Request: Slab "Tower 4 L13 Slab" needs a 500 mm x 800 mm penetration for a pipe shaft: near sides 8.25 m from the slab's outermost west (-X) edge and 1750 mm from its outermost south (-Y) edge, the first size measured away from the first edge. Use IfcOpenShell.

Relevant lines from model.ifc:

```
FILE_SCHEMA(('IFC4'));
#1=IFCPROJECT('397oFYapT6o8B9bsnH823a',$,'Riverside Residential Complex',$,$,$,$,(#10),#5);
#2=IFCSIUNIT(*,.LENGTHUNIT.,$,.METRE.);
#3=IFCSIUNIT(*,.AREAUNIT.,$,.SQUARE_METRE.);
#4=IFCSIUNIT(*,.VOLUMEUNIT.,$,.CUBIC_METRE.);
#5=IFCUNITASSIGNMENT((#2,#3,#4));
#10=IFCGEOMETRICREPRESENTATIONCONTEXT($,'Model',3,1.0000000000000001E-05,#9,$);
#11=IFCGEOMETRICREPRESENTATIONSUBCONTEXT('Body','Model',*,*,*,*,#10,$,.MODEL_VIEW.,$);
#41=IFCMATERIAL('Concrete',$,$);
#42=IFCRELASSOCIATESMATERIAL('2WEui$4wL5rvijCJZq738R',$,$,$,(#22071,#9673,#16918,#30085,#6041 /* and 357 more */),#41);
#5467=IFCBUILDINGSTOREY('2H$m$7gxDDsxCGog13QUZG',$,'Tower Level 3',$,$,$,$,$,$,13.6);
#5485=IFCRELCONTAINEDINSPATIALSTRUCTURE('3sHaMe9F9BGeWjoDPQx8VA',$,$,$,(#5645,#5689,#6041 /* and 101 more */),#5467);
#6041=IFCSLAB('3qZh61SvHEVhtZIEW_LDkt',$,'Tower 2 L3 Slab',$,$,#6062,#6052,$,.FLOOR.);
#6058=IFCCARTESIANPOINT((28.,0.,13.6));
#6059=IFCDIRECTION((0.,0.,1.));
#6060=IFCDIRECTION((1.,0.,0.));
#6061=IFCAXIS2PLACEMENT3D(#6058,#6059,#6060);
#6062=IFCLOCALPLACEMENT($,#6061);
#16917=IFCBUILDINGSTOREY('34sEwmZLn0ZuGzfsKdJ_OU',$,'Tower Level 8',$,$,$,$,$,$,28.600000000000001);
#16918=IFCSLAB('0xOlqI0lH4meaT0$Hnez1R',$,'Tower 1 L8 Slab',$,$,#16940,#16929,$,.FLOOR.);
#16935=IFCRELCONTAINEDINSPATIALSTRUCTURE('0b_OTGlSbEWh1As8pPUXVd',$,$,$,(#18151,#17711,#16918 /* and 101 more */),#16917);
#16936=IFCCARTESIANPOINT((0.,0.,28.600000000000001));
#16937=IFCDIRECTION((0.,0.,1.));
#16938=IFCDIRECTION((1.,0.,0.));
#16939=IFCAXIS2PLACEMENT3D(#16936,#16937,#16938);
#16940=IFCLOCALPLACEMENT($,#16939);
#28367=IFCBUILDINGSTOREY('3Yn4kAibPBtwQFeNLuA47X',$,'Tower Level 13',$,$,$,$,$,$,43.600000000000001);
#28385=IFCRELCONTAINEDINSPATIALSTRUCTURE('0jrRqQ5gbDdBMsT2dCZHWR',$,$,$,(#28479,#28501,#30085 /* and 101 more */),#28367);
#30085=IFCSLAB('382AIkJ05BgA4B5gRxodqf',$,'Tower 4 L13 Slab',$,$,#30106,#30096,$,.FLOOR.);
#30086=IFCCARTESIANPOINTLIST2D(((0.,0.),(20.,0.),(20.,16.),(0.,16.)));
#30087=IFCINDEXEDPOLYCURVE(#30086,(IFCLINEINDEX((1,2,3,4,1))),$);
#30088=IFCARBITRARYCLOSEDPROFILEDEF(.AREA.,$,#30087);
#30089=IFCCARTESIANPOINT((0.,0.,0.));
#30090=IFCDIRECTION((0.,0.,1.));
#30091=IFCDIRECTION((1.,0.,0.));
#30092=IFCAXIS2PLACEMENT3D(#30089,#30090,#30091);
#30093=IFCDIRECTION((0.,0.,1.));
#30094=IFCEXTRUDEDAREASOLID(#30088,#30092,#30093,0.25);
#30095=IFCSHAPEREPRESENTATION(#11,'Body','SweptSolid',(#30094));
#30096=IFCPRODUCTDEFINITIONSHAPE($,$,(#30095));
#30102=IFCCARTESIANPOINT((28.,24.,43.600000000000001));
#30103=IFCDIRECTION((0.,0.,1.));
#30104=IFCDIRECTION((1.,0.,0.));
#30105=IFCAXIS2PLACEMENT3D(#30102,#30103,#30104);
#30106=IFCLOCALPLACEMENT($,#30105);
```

```python
import numpy as np
import ifcopenshell
import ifcopenshell.api.feature
import ifcopenshell.api.geometry
import ifcopenshell.api.root
import ifcopenshell.geom
import ifcopenshell.util.placement
import ifcopenshell.util.representation
import ifcopenshell.util.shape
import ifcopenshell.util.unit

model = ifcopenshell.open("model.ifc")
unit_scale = ifcopenshell.util.unit.calculate_unit_scale(model)
settings = ifcopenshell.geom.settings()


def volume(element):
    """Net volume in cubic metres, openings subtracted."""
    shape = ifcopenshell.geom.create_shape(settings, element)
    return ifcopenshell.util.shape.get_volume(shape.geometry)


slab = model.by_id(30085)
before = volume(slab)

# Extent in the slab's own axes, in metres. The edges named are its -X and -Y sides.
slab_shape = ifcopenshell.geom.create_shape(settings, slab)
vertices = ifcopenshell.util.shape.get_vertices(slab_shape.geometry)
x_min, y_min, bottom = vertices.min(axis=0)
top = vertices[:, 2].max()

opening = ifcopenshell.api.root.create_entity(model, ifc_class="IfcOpeningElement", name="Pipe shaft opening", predefined_type="OPENING")
context = ifcopenshell.util.representation.get_context(model, "Model", "Body", "MODEL_VIEW")
width, depth = 0.5, 0.8
outline = [(0.0, 0.0), (width, 0.0), (width, depth), (0.0, depth), (0.0, 0.0)]
# Overshoot both faces by 50 mm so the cut is clean.
shape = ifcopenshell.api.geometry.add_slab_representation(
    model, context=context, depth=top - bottom + 0.1, polyline=outline
)
ifcopenshell.api.geometry.assign_representation(model, product=opening, representation=shape)

matrix = ifcopenshell.util.placement.get_local_placement(slab.ObjectPlacement)
matrix[:, 3] = matrix @ np.append(np.array([x_min + 8.25, y_min + 1.75, bottom - 0.05]) / unit_scale, 1.0)
ifcopenshell.api.geometry.edit_object_placement(model, product=opening, matrix=matrix, is_si=False)
ifcopenshell.api.feature.add_feature(model, feature=opening, element=slab)

after = volume(slab)

print(f"slab volume {before:.3f} -> {after:.3f} m3")

model.write("model-out.ifc")
```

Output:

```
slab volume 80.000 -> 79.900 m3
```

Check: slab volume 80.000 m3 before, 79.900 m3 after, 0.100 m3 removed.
